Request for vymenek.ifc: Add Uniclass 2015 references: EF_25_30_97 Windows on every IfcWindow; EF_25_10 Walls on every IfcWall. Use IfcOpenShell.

First a look at what the model holds.

```python
import ifcopenshell

model = ifcopenshell.open("vymenek.ifc")
print(model.schema)
print("classifications:", [c.Name for c in model.by_type("IfcClassification")])
for ifc_class in ("IfcDoor", "IfcRoof", "IfcStair", "IfcWall", "IfcWindow"):
    print(ifc_class, len(model.by_type(ifc_class)))
```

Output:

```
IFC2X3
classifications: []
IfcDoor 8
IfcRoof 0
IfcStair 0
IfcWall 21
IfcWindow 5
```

```python
import ifcopenshell
import ifcopenshell.api.classification

model = ifcopenshell.open("vymenek.ifc")

# IFC2X3 requires Source and Edition and has no link from the project to the system.
system = model.create_entity("IfcClassification", Source="NBS", Edition="2015", Name="Uniclass 2015")

codes = {
    "IfcWindow": ("EF_25_30_97", "Windows"),
    "IfcWall": ("EF_25_10", "Walls"),
}
for ifc_class, (code, name) in codes.items():
    products = model.by_type(ifc_class)
    ifcopenshell.api.classification.add_reference(
        model, products=products, classification=system, identification=code, name=name
    )
    print(code, len(products))

model.write("vymenek_rev.ifc")
```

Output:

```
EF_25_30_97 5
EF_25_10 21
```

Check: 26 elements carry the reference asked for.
